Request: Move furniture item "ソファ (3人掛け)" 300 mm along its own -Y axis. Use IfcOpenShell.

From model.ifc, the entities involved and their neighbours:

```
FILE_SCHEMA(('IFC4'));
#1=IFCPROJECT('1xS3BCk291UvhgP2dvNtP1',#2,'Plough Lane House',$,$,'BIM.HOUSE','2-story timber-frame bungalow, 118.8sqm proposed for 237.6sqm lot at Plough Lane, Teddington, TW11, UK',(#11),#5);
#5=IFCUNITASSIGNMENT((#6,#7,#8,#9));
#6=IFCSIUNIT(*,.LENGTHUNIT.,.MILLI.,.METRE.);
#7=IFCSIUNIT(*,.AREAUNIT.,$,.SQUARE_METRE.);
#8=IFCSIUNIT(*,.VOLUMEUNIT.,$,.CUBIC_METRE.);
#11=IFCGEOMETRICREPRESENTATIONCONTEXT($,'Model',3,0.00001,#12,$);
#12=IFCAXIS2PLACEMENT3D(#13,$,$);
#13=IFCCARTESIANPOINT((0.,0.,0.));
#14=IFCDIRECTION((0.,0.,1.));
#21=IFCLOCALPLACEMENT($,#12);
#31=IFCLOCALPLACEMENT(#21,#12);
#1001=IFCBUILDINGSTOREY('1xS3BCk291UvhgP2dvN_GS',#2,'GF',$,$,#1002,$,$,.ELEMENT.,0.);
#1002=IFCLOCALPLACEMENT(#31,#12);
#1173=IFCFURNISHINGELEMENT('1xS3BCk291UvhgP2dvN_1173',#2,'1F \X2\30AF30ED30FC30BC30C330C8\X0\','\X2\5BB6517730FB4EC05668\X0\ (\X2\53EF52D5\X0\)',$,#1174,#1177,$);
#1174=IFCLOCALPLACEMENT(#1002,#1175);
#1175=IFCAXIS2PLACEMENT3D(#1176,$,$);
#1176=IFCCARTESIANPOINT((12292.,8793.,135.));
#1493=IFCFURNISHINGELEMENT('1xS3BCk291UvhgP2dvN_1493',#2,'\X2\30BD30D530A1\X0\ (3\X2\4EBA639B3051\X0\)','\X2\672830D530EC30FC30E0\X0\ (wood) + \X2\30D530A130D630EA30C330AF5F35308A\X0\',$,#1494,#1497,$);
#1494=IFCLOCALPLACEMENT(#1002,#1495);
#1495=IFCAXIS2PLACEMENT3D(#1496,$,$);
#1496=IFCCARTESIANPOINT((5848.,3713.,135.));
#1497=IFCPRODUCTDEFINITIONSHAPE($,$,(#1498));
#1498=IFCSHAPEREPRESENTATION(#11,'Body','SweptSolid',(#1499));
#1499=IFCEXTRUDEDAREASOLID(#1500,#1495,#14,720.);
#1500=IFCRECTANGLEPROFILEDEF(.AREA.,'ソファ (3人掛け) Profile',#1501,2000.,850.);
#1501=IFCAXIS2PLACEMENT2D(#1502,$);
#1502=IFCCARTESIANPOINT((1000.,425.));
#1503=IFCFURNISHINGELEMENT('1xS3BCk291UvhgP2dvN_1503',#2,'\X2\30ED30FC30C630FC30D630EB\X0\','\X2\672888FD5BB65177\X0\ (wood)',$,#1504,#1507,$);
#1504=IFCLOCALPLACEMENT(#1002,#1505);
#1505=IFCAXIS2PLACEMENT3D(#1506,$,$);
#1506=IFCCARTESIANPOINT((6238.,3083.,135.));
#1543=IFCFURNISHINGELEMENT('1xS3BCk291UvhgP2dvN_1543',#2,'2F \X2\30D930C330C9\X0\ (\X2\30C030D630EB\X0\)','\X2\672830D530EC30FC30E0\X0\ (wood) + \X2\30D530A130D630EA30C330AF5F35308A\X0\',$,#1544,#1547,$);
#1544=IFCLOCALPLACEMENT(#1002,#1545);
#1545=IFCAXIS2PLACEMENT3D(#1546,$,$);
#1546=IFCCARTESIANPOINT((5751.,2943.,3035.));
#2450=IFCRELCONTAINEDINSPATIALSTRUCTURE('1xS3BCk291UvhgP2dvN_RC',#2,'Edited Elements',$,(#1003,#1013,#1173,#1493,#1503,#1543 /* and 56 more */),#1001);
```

```python
import ifcopenshell
import ifcopenshell.api.geometry
import ifcopenshell.util.placement
import ifcopenshell.util.unit

model = ifcopenshell.open("model.ifc")
unit_scale = ifcopenshell.util.unit.calculate_unit_scale(model)

item = model.by_guid("1xS3BCk291UvhgP2dvN_1493")
matrix = ifcopenshell.util.placement.get_local_placement(item.ObjectPlacement)
matrix[:3, 3] -= matrix[:3, 1] * 0.3 / unit_scale
ifcopenshell.api.geometry.edit_object_placement(model, product=item, matrix=matrix, is_si=False)

print(ifcopenshell.util.placement.get_local_placement(item.ObjectPlacement).round(3) + 0.0)

model.write("model_rev.ifc")
```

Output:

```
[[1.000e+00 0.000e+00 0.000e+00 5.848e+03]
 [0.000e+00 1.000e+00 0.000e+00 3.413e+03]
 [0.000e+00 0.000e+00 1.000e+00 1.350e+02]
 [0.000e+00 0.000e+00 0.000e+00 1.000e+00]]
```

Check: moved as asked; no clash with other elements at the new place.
